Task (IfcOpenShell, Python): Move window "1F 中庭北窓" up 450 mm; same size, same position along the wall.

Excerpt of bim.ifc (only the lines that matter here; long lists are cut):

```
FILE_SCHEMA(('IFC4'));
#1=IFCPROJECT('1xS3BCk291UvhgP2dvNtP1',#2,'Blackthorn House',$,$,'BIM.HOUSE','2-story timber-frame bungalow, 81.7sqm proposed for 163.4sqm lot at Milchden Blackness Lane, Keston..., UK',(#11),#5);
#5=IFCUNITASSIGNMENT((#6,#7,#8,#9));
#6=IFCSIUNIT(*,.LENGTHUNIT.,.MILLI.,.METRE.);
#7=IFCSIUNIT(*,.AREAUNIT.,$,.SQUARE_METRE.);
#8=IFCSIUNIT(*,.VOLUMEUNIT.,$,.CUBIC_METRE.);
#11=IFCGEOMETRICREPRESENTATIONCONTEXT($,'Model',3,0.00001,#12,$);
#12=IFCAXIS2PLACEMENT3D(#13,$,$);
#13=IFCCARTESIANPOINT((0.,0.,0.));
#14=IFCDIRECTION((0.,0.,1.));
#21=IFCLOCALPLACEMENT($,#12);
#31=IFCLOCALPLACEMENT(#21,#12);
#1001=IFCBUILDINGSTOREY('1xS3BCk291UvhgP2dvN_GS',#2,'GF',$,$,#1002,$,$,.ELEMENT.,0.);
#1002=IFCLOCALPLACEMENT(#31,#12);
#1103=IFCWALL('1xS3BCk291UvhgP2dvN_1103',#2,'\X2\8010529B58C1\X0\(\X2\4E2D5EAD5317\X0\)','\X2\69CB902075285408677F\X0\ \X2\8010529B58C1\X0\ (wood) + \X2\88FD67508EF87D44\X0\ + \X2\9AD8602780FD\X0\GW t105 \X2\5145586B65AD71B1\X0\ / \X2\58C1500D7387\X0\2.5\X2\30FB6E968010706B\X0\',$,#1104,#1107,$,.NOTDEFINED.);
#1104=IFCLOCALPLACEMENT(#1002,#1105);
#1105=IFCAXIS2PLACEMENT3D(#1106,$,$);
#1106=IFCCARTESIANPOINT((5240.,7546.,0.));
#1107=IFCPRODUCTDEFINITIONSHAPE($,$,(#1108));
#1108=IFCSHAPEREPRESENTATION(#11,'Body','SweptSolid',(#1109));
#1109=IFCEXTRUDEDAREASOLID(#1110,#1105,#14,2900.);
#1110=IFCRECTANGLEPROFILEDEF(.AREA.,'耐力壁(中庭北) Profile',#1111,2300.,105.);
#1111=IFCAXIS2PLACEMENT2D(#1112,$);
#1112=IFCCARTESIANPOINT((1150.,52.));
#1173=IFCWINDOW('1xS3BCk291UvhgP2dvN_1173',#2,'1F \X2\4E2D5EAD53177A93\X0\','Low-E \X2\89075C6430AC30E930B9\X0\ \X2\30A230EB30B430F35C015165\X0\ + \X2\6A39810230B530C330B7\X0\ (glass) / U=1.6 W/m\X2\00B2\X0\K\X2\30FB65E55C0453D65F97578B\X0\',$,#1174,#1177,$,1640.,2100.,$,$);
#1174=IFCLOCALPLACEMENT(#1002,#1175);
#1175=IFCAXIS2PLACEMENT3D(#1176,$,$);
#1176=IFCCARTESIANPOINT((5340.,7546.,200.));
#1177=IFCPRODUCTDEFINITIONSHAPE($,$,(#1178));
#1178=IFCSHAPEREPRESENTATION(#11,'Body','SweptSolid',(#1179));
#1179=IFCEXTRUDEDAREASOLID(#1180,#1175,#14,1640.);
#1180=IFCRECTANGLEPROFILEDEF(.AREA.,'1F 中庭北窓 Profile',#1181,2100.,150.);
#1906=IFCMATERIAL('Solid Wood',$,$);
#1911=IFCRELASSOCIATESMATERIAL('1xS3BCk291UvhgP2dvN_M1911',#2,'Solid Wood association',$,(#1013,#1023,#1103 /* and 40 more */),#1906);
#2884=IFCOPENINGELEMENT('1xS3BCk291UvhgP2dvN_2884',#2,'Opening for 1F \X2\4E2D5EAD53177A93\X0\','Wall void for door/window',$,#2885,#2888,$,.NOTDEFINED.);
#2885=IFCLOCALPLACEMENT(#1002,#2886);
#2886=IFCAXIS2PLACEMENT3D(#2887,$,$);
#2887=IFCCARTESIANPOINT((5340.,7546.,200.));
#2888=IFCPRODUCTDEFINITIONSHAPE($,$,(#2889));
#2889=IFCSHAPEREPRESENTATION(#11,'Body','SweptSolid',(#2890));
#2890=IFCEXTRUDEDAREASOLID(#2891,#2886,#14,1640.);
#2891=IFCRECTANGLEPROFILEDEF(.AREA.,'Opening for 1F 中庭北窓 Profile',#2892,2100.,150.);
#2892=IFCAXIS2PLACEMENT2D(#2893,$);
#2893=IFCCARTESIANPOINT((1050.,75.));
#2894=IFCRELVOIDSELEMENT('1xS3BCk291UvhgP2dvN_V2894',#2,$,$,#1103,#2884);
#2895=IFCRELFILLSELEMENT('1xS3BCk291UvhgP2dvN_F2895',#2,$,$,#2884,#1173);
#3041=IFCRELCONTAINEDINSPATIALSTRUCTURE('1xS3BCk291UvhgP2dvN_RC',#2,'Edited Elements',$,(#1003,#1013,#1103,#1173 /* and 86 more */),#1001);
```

```python
import numpy as np
import ifcopenshell
import ifcopenshell.api.geometry
import ifcopenshell.util.placement
import ifcopenshell.util.unit

model = ifcopenshell.open("bim.ifc")
unit_scale = ifcopenshell.util.unit.calculate_unit_scale(model)

window = model.by_guid("1xS3BCk291UvhgP2dvN_1173")
opening = window.FillsVoids[0].RelatingOpeningElement
dz = 0.45 / unit_scale

shift = np.array([0.0, 0.0, dz])
# The window is not placed relative to its opening, so move both.
for product in (opening, window):
    matrix = ifcopenshell.util.placement.get_local_placement(product.ObjectPlacement)
    matrix[:3, 3] += shift
    ifcopenshell.api.geometry.edit_object_placement(model, product=product, matrix=matrix, is_si=False)

print(f"moved by {dz * unit_scale:+.3f} m")

model.write("bim_edited.ifc")
```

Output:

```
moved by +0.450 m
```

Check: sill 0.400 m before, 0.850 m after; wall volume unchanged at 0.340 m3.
